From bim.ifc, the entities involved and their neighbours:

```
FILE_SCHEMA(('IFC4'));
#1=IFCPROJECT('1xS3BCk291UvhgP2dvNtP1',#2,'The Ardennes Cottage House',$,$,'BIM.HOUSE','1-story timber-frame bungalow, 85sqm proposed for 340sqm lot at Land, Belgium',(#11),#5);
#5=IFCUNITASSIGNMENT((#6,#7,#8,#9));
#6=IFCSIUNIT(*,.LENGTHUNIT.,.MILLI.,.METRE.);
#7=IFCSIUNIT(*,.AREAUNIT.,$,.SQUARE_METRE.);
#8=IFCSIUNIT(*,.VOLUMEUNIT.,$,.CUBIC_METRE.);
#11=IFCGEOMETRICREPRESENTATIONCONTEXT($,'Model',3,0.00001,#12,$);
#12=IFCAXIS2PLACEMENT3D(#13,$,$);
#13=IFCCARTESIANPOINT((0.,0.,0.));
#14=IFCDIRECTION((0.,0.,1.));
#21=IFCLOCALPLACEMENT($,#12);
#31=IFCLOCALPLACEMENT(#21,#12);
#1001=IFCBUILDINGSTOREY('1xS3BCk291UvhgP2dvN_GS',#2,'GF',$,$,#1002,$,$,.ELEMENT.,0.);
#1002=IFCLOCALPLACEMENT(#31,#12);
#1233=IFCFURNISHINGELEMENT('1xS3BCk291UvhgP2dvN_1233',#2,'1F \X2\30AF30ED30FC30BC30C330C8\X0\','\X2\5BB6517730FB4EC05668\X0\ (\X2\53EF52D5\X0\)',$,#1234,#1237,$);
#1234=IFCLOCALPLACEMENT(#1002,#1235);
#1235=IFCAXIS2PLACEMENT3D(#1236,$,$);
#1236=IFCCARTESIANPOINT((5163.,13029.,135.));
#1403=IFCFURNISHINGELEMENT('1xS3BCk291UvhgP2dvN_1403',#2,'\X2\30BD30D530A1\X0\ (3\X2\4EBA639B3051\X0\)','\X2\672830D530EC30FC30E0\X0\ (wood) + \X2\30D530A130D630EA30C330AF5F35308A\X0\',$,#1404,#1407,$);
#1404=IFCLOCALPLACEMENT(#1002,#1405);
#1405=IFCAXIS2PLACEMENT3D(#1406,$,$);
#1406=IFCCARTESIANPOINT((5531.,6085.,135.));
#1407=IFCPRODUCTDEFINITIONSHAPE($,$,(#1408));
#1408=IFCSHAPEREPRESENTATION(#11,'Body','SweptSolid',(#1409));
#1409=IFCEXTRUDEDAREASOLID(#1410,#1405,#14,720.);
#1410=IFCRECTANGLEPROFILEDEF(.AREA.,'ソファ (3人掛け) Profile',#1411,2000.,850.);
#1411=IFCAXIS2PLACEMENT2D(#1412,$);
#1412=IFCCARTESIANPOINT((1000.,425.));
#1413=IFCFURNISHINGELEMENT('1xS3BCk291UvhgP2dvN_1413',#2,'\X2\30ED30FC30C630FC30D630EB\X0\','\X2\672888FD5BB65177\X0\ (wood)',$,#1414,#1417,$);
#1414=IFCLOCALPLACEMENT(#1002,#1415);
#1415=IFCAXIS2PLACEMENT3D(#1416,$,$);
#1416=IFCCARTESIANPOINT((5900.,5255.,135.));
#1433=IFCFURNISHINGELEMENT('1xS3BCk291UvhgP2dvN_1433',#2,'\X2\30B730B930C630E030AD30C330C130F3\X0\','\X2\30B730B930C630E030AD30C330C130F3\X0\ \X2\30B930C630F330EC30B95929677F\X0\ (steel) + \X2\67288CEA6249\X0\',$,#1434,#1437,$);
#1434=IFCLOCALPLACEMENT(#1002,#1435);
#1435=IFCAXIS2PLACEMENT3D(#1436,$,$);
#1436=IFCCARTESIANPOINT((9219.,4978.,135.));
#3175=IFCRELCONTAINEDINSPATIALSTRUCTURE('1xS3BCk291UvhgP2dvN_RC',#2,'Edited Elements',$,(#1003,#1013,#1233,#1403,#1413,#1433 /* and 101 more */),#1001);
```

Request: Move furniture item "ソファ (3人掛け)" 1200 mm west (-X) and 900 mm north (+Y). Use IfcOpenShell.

```python
import ifcopenshell
import ifcopenshell.api.geometry
import ifcopenshell.util.placement

model = ifcopenshell.open("bim.ifc")

item = model.by_guid("1xS3BCk291UvhgP2dvN_1403")
matrix = ifcopenshell.util.placement.get_local_placement(item.ObjectPlacement)
matrix[0, 3] -= 1200.0
matrix[1, 3] += 900.0
ifcopenshell.api.geometry.edit_object_placement(model, product=item, matrix=matrix, is_si=False)

print(ifcopenshell.util.placement.get_local_placement(item.ObjectPlacement).round(3) + 0.0)

model.write("bim_rev.ifc")
```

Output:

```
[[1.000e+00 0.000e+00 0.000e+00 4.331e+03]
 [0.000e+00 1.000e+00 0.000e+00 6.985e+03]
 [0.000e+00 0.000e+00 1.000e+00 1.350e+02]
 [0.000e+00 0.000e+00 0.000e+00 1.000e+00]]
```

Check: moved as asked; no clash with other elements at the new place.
